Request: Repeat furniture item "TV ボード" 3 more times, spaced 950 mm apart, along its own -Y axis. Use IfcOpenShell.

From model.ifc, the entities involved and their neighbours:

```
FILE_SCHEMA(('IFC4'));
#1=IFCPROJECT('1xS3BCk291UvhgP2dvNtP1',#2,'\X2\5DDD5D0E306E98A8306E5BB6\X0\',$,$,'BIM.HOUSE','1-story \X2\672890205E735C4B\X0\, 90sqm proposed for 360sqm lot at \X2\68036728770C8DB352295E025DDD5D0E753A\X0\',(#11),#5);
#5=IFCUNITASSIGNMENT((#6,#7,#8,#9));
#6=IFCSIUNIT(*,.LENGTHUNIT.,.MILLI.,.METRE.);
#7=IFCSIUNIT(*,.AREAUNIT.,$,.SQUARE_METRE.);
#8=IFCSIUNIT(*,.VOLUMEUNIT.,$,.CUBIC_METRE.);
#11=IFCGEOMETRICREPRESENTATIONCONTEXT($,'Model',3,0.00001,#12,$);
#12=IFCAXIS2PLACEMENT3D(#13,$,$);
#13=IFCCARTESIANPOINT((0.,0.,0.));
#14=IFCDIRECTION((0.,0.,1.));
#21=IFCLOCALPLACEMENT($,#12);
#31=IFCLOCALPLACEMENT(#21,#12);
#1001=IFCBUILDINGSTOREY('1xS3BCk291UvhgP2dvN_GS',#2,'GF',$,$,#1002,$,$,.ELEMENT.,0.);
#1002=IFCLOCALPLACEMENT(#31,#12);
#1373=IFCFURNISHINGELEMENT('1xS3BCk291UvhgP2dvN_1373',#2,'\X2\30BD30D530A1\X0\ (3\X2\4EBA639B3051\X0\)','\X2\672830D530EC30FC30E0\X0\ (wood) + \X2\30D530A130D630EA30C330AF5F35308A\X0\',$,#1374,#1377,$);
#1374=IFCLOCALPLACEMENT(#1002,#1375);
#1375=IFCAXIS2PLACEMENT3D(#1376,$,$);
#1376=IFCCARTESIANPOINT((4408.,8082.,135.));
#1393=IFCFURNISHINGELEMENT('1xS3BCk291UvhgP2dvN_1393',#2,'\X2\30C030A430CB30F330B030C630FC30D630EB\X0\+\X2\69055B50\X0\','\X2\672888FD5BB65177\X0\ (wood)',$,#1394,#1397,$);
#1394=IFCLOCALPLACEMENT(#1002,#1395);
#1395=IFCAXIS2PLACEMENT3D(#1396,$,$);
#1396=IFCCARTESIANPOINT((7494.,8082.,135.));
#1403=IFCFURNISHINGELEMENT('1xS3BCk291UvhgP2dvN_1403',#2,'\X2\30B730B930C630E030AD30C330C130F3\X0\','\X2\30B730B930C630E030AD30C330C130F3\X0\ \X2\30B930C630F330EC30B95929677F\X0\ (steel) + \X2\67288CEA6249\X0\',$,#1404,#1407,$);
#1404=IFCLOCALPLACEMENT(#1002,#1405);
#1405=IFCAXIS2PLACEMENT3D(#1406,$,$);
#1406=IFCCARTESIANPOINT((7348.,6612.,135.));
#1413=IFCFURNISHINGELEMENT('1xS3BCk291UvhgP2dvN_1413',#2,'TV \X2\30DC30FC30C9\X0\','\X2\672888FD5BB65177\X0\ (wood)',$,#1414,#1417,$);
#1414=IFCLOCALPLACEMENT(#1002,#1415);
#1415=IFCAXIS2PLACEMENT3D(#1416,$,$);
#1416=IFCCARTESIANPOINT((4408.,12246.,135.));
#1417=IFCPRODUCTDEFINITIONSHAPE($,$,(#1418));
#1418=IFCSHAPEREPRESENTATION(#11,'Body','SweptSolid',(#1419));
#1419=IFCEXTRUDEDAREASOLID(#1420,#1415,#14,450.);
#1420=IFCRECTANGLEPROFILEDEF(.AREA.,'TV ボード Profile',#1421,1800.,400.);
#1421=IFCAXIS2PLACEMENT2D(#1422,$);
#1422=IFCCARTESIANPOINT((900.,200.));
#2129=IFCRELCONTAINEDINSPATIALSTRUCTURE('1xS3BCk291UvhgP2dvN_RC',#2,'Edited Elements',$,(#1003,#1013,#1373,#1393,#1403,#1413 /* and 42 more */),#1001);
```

```python
import ifcopenshell
import ifcopenshell.api.geometry
import ifcopenshell.api.root
import ifcopenshell.util.element
import ifcopenshell.util.placement
import ifcopenshell.util.unit

model = ifcopenshell.open("model.ifc")
unit_scale = ifcopenshell.util.unit.calculate_unit_scale(model)


def reuse_history(source, copy):
    """copy_class also copies each property set's owner history, people and application; keep the originals."""
    for rel in copy.IsDefinedBy:
        if rel.is_a("IfcRelDefinesByProperties") and (history := rel.RelatingPropertyDefinition.OwnerHistory):
            rel.RelatingPropertyDefinition.OwnerHistory = source.OwnerHistory
            ifcopenshell.util.element.remove_deep2(model, history)


source = model.by_guid("1xS3BCk291UvhgP2dvN_1413")
base = ifcopenshell.util.placement.get_local_placement(source.ObjectPlacement)
step = -base[:3, 1] * 0.95 / unit_scale

for i in range(1, 4):
    copy = ifcopenshell.api.root.copy_class(model, product=source)
    copy.Representation = ifcopenshell.util.element.copy_deep(
        model, source.Representation, exclude=["IfcGeometricRepresentationContext", "IfcRepresentationMap"]
    )
    reuse_history(source, copy)
    matrix = base.copy()
    matrix[:3, 3] += i * step
    print("added at", matrix[:3, 3].round(3) + 0.0)
    ifcopenshell.api.geometry.edit_object_placement(model, product=copy, matrix=matrix, is_si=False)

model.write("model_edited.ifc")
```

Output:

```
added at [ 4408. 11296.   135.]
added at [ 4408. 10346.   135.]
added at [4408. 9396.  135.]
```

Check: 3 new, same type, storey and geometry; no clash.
